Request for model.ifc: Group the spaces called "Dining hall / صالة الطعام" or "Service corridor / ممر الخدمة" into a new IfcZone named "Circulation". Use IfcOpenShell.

First a look at what the model holds.

```python
import ifcopenshell

model = ifcopenshell.open("model.ifc")
print(model.schema)
seen = {}
for space in model.by_type("IfcSpace"):
    seen[space.LongName] = seen.get(space.LongName, 0) + 1
for name, count in sorted(seen.items(), key=str):
    print(count, "x", name)
print("zones:", [z.Name for z in model.by_type("IfcZone")][:20])
```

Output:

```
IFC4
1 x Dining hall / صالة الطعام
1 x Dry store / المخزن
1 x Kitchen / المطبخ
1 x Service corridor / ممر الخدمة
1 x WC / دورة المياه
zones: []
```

```python
import ifcopenshell
import ifcopenshell.api.group
import ifcopenshell.api.root

model = ifcopenshell.open("model.ifc")

names = {"Dining hall / صالة الطعام", "Service corridor / ممر الخدمة"}
spaces = [s for s in model.by_type("IfcSpace") if s.LongName in names]

zone = ifcopenshell.api.root.create_entity(model, ifc_class="IfcZone", name="Circulation")
ifcopenshell.api.group.assign_group(model, products=spaces, group=zone)
print(len(spaces), "spaces in", zone.Name)

model.write("model-out.ifc")
```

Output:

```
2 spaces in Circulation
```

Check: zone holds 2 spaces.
